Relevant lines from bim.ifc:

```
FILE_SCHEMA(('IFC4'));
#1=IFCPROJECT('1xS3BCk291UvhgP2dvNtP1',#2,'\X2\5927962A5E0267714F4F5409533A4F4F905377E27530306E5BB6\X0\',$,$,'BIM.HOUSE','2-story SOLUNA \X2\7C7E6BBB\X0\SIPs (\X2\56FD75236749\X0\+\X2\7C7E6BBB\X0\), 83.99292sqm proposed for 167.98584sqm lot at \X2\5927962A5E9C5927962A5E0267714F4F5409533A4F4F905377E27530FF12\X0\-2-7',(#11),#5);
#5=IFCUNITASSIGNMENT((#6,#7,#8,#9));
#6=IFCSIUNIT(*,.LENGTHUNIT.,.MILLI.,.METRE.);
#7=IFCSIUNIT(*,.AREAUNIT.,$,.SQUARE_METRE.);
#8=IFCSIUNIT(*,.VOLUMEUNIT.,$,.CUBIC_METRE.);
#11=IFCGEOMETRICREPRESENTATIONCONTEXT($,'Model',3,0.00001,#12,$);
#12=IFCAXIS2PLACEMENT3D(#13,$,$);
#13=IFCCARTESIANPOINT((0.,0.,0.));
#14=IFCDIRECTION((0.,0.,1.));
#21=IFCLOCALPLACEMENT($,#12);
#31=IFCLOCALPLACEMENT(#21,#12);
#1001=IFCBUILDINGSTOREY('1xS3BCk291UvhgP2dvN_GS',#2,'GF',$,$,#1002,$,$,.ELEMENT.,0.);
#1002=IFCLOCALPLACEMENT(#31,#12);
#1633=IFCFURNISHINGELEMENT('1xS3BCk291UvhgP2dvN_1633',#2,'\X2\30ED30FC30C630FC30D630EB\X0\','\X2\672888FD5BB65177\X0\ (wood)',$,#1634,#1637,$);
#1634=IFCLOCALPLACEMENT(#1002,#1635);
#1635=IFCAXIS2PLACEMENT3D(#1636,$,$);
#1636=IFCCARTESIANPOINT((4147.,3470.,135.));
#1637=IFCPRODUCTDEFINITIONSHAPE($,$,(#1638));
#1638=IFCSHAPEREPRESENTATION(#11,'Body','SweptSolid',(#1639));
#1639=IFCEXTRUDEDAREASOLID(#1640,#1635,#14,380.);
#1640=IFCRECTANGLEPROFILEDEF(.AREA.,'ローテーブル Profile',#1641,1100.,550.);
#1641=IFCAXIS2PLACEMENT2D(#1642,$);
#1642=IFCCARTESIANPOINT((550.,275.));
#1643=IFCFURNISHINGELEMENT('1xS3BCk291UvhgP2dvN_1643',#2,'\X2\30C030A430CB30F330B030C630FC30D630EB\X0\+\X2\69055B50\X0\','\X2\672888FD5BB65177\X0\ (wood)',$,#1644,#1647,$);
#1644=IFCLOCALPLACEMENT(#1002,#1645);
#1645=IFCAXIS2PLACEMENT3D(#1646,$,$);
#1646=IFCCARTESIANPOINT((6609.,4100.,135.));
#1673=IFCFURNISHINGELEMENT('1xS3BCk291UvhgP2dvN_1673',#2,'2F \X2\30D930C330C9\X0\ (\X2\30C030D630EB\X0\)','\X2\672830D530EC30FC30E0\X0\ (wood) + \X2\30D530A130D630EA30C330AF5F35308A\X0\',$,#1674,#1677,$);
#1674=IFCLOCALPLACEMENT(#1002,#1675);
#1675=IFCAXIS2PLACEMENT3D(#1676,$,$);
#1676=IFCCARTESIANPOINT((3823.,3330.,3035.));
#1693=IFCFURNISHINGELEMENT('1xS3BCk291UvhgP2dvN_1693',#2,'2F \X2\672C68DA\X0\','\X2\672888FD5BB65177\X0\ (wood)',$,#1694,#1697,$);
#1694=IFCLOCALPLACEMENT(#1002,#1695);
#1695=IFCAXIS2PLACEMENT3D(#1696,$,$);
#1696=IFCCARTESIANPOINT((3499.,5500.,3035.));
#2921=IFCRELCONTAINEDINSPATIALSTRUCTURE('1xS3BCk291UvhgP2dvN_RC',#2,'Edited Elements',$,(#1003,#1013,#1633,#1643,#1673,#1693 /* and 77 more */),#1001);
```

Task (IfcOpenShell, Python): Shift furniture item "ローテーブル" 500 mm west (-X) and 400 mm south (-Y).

```python
import ifcopenshell
import ifcopenshell.api.geometry
import ifcopenshell.util.placement
import ifcopenshell.util.unit

model = ifcopenshell.open("bim.ifc")
unit_scale = ifcopenshell.util.unit.calculate_unit_scale(model)

item = model.by_guid("1xS3BCk291UvhgP2dvN_1633")
matrix = ifcopenshell.util.placement.get_local_placement(item.ObjectPlacement)
matrix[0, 3] -= 0.5 / unit_scale
matrix[1, 3] -= 0.4 / unit_scale
ifcopenshell.api.geometry.edit_object_placement(model, product=item, matrix=matrix, is_si=False)

print(ifcopenshell.util.placement.get_local_placement(item.ObjectPlacement).round(3) + 0.0)

model.write("bim_updated.ifc")
```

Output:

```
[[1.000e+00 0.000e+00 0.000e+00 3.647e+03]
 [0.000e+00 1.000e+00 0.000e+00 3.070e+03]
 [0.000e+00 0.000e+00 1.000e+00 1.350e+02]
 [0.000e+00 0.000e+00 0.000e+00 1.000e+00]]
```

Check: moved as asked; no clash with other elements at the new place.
